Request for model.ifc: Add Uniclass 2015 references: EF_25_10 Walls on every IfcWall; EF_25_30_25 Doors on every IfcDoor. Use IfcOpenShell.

First a look at what the model holds.

```python
import ifcopenshell

model = ifcopenshell.open("model.ifc")
print(model.schema)
print("classifications:", [c.Name for c in model.by_type("IfcClassification")])
for ifc_class in ("IfcDoor", "IfcRoof", "IfcStair", "IfcWall", "IfcWindow"):
    print(ifc_class, len(model.by_type(ifc_class)))
```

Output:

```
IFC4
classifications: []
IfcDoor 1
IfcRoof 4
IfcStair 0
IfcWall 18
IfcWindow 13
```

```python
import ifcopenshell
import ifcopenshell.api.classification

model = ifcopenshell.open("model.ifc")

system = ifcopenshell.api.classification.add_classification(model, classification="Uniclass 2015")

codes = {
    "IfcWall": ("EF_25_10", "Walls"),
    "IfcDoor": ("EF_25_30_25", "Doors"),
}
for ifc_class, (code, name) in codes.items():
    products = model.by_type(ifc_class)
    ifcopenshell.api.classification.add_reference(
        model, products=products, classification=system, identification=code, name=name
    )
    print(code, len(products))

model.write("model-out.ifc")
```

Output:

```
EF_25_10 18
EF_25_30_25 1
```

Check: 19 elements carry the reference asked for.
